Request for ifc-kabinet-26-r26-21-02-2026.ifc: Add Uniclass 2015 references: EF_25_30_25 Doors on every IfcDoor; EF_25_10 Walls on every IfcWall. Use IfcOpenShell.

First a look at what the model holds.

```python
import ifcopenshell

model = ifcopenshell.open("ifc-kabinet-26-r26-21-02-2026.ifc")
print(model.schema)
print("classifications:", [c.Name for c in model.by_type("IfcClassification")])
for ifc_class in ("IfcDoor", "IfcRoof", "IfcStair", "IfcWall", "IfcWindow"):
    print(ifc_class, len(model.by_type(ifc_class)))
```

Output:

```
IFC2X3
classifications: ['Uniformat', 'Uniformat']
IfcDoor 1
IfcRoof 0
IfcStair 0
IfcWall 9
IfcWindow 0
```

```python
import ifcopenshell
import ifcopenshell.api.classification

model = ifcopenshell.open("ifc-kabinet-26-r26-21-02-2026.ifc")

# IFC2X3 requires Source and Edition and has no link from the project to the system.
system = model.create_entity("IfcClassification", Source="NBS", Edition="2015", Name="Uniclass 2015")

codes = {
    "IfcDoor": ("EF_25_30_25", "Doors"),
    "IfcWall": ("EF_25_10", "Walls"),
}
for ifc_class, (code, name) in codes.items():
    products = model.by_type(ifc_class)
    ifcopenshell.api.classification.add_reference(
        model, products=products, classification=system, identification=code, name=name
    )
    print(code, len(products))

model.write("ifc-kabinet-26-r26-21-02-2026_updated.ifc")
```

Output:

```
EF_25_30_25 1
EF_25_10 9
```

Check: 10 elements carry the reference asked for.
